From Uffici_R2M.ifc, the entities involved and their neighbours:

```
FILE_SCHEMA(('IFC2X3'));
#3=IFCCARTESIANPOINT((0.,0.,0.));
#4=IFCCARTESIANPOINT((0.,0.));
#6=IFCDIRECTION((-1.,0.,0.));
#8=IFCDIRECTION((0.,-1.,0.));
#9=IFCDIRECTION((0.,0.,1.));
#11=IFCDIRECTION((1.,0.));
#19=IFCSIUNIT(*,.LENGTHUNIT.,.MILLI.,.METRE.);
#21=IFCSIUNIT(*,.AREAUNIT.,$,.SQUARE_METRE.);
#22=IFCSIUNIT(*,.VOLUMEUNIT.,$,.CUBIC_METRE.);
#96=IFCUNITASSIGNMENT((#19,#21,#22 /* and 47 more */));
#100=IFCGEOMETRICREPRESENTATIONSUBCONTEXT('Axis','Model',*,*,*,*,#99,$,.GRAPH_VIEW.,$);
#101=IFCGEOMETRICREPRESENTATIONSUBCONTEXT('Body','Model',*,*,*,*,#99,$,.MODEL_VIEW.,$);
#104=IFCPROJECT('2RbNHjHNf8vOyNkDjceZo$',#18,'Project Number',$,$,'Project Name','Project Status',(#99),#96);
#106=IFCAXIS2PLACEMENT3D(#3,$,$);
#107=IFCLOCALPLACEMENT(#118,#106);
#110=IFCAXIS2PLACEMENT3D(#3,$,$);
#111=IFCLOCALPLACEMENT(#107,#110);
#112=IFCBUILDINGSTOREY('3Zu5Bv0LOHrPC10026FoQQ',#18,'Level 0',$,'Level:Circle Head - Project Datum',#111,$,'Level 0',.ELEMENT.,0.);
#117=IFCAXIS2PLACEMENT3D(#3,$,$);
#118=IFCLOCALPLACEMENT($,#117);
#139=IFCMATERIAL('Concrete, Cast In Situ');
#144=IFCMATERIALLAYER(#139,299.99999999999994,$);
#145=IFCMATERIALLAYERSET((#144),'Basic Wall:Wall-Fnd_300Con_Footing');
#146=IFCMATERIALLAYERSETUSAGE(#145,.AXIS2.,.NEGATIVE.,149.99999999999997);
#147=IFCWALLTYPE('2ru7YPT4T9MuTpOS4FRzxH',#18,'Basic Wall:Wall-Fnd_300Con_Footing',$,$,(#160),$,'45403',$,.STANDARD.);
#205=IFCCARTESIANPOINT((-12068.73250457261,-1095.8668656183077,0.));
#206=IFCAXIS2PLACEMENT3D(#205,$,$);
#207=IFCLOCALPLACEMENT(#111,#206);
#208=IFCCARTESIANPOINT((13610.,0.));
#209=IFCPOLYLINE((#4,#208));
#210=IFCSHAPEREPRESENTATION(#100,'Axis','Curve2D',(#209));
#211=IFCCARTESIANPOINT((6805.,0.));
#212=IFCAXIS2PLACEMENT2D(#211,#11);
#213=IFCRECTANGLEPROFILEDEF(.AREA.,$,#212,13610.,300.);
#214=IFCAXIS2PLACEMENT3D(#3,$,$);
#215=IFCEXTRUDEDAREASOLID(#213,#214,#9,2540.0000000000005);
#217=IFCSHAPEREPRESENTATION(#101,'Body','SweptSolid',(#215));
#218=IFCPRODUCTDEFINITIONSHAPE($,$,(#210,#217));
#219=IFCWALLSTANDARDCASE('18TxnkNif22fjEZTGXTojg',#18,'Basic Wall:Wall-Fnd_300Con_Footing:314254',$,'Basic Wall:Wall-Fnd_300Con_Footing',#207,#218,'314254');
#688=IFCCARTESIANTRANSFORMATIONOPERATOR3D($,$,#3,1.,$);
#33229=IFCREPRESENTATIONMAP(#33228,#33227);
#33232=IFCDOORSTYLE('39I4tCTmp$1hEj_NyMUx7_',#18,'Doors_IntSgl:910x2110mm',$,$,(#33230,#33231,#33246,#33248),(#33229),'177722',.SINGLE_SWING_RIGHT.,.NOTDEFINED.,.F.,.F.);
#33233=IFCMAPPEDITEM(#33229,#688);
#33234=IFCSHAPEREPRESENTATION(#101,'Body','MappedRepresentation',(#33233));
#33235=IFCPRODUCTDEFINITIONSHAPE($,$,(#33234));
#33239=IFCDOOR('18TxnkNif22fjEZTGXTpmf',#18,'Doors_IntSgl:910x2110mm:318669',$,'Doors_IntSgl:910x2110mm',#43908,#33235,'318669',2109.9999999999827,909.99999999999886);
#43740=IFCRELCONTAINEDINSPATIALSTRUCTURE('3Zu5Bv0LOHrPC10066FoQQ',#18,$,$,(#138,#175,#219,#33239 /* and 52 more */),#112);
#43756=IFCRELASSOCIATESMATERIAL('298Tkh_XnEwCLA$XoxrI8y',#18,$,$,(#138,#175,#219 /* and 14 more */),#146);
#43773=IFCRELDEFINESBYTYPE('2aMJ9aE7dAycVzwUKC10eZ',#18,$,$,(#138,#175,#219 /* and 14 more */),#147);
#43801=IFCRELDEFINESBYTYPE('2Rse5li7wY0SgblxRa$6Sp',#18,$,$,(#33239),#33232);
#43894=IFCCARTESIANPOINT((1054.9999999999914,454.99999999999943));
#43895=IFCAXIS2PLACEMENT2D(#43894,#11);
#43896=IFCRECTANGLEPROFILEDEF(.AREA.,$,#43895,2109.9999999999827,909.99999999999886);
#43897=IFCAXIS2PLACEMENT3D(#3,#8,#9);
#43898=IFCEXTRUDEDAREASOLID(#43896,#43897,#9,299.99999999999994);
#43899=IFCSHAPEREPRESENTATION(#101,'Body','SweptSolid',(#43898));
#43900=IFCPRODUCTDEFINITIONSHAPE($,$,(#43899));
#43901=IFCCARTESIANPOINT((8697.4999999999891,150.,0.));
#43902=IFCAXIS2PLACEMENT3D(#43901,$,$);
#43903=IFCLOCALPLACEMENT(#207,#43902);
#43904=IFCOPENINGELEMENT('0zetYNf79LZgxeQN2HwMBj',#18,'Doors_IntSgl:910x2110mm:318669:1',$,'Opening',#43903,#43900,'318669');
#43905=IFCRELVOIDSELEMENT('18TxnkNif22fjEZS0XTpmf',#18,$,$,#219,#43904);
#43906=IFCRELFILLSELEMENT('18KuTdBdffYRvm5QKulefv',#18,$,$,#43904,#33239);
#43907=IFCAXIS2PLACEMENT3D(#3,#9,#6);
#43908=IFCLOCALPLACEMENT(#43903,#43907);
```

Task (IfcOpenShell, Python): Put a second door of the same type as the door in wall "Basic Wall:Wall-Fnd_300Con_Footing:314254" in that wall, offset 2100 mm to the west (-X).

```python
import ifcopenshell
import ifcopenshell.api.feature
import ifcopenshell.api.geometry
import ifcopenshell.api.root
import ifcopenshell.geom
import ifcopenshell.util.element
import ifcopenshell.util.placement
import ifcopenshell.util.shape
import ifcopenshell.util.unit

model = ifcopenshell.open("Uffici_R2M.ifc")
unit_scale = ifcopenshell.util.unit.calculate_unit_scale(model)
settings = ifcopenshell.geom.settings()


def volume(element):
    """Net volume in cubic metres, openings subtracted."""
    shape = ifcopenshell.geom.create_shape(settings, element)
    return ifcopenshell.util.shape.get_volume(shape.geometry)


def reuse_history(source, copy):
    """copy_class also copies each property set's owner history, people and application; keep the originals."""
    for rel in copy.IsDefinedBy:
        if rel.is_a("IfcRelDefinesByProperties") and (history := rel.RelatingPropertyDefinition.OwnerHistory):
            rel.RelatingPropertyDefinition.OwnerHistory = source.OwnerHistory
            ifcopenshell.util.element.remove_deep2(model, history)


door = model.by_guid("18TxnkNif22fjEZTGXTpmf")
opening = door.FillsVoids[0].RelatingOpeningElement
wall = opening.VoidsElements[0].RelatingBuildingElement
before = volume(wall)
shift = ifcopenshell.util.placement.get_local_placement(wall.ObjectPlacement)[:3, 0] * -2.1 / unit_scale

# copy_class copies the void relationship, type, container and properties, but no geometry.
new_opening = ifcopenshell.api.root.copy_class(model, product=opening)
new_opening.Representation = ifcopenshell.util.element.copy_deep(
    model, opening.Representation, exclude=["IfcGeometricRepresentationContext", "IfcRepresentationMap"]
)
new_opening.Name = "Doors_IntSgl:910x2110mm"
new_opening.Tag = None
new_door = ifcopenshell.api.root.copy_class(model, product=door)
new_door.Representation = ifcopenshell.util.element.copy_deep(
    model, door.Representation, exclude=["IfcGeometricRepresentationContext", "IfcRepresentationMap"]
)
new_door.Name = "Doors_IntSgl:910x2110mm"
new_door.Tag = None
reuse_history(door, new_door)
fills = ifcopenshell.api.feature.add_filling(model, opening=new_opening, element=new_door)
fills.OwnerHistory = new_door.OwnerHistory  # required in IFC2X3

for old, new in ((opening, new_opening), (door, new_door)):
    matrix = ifcopenshell.util.placement.get_local_placement(old.ObjectPlacement)
    matrix[:3, 3] += shift
    ifcopenshell.api.geometry.edit_object_placement(model, product=new, matrix=matrix, is_si=False)

after = volume(wall)

print(f"wall volume {before:.3f} -> {after:.3f} m3")

model.write("Uffici_R2M_updated.ifc")
```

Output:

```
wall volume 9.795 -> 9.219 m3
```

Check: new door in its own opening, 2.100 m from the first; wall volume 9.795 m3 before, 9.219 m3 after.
